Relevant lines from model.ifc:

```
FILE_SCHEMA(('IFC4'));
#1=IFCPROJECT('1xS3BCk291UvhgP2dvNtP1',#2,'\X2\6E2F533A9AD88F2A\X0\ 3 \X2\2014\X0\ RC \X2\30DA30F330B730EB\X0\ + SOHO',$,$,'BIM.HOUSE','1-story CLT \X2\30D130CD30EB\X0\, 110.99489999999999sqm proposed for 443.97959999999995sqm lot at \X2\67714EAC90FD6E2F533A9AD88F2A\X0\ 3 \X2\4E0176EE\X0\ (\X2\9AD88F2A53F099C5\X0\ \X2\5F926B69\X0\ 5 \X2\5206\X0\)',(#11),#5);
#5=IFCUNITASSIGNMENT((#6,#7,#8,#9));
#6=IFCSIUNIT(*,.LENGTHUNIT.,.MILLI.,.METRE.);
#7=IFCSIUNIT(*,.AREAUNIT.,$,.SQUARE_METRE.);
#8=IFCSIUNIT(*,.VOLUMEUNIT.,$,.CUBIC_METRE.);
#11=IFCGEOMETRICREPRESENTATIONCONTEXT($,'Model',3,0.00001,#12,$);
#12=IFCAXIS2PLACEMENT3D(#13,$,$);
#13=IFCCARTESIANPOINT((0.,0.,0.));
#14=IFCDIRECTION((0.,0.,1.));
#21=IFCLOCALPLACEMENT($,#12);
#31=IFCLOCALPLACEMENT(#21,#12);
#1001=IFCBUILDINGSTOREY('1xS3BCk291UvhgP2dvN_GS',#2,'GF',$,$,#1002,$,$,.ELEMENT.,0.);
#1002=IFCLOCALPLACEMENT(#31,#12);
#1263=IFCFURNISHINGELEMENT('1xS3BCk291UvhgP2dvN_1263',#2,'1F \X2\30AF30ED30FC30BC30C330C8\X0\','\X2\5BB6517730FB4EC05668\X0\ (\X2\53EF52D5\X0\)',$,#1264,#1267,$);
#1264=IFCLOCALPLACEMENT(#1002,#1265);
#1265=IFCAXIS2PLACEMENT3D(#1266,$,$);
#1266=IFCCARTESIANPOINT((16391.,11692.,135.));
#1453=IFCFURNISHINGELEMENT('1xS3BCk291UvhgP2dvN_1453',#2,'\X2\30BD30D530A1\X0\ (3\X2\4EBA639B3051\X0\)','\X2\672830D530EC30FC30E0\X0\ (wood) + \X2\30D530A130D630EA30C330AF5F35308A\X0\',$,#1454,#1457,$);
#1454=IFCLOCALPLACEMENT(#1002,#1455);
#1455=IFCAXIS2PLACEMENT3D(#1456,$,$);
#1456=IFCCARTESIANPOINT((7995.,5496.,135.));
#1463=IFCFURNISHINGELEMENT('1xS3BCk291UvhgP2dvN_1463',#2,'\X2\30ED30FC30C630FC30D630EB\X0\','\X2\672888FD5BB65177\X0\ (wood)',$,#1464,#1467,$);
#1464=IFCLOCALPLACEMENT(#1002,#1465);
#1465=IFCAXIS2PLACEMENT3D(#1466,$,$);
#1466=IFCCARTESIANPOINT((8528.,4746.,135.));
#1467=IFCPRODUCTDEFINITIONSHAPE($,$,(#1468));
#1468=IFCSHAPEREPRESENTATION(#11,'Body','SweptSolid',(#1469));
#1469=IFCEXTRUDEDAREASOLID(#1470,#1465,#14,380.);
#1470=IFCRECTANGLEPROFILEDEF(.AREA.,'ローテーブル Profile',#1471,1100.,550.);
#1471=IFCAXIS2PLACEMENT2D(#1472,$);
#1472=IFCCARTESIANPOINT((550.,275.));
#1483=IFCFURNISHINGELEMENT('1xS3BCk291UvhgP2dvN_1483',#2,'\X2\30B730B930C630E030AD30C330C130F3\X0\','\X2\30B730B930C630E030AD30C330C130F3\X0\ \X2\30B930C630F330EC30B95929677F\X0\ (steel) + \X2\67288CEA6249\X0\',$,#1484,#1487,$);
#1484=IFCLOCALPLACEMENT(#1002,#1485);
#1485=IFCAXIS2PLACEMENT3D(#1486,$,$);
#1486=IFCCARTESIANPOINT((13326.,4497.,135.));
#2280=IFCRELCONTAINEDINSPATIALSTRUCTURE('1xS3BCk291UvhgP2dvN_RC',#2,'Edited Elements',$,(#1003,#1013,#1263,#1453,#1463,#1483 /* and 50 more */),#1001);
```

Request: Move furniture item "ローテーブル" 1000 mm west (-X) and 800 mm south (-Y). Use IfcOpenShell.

```python
import ifcopenshell
import ifcopenshell.api.geometry
import ifcopenshell.util.placement
import ifcopenshell.util.unit

model = ifcopenshell.open("model.ifc")
unit_scale = ifcopenshell.util.unit.calculate_unit_scale(model)

item = model.by_guid("1xS3BCk291UvhgP2dvN_1463")
matrix = ifcopenshell.util.placement.get_local_placement(item.ObjectPlacement)
matrix[0, 3] -= 1 / unit_scale
matrix[1, 3] -= 0.8 / unit_scale
ifcopenshell.api.geometry.edit_object_placement(model, product=item, matrix=matrix, is_si=False)

print(ifcopenshell.util.placement.get_local_placement(item.ObjectPlacement).round(3) + 0.0)

model.write("model_rev.ifc")
```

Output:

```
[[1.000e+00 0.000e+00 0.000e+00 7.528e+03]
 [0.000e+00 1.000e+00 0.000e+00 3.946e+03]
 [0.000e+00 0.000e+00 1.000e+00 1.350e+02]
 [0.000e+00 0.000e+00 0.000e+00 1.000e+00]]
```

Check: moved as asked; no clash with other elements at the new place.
